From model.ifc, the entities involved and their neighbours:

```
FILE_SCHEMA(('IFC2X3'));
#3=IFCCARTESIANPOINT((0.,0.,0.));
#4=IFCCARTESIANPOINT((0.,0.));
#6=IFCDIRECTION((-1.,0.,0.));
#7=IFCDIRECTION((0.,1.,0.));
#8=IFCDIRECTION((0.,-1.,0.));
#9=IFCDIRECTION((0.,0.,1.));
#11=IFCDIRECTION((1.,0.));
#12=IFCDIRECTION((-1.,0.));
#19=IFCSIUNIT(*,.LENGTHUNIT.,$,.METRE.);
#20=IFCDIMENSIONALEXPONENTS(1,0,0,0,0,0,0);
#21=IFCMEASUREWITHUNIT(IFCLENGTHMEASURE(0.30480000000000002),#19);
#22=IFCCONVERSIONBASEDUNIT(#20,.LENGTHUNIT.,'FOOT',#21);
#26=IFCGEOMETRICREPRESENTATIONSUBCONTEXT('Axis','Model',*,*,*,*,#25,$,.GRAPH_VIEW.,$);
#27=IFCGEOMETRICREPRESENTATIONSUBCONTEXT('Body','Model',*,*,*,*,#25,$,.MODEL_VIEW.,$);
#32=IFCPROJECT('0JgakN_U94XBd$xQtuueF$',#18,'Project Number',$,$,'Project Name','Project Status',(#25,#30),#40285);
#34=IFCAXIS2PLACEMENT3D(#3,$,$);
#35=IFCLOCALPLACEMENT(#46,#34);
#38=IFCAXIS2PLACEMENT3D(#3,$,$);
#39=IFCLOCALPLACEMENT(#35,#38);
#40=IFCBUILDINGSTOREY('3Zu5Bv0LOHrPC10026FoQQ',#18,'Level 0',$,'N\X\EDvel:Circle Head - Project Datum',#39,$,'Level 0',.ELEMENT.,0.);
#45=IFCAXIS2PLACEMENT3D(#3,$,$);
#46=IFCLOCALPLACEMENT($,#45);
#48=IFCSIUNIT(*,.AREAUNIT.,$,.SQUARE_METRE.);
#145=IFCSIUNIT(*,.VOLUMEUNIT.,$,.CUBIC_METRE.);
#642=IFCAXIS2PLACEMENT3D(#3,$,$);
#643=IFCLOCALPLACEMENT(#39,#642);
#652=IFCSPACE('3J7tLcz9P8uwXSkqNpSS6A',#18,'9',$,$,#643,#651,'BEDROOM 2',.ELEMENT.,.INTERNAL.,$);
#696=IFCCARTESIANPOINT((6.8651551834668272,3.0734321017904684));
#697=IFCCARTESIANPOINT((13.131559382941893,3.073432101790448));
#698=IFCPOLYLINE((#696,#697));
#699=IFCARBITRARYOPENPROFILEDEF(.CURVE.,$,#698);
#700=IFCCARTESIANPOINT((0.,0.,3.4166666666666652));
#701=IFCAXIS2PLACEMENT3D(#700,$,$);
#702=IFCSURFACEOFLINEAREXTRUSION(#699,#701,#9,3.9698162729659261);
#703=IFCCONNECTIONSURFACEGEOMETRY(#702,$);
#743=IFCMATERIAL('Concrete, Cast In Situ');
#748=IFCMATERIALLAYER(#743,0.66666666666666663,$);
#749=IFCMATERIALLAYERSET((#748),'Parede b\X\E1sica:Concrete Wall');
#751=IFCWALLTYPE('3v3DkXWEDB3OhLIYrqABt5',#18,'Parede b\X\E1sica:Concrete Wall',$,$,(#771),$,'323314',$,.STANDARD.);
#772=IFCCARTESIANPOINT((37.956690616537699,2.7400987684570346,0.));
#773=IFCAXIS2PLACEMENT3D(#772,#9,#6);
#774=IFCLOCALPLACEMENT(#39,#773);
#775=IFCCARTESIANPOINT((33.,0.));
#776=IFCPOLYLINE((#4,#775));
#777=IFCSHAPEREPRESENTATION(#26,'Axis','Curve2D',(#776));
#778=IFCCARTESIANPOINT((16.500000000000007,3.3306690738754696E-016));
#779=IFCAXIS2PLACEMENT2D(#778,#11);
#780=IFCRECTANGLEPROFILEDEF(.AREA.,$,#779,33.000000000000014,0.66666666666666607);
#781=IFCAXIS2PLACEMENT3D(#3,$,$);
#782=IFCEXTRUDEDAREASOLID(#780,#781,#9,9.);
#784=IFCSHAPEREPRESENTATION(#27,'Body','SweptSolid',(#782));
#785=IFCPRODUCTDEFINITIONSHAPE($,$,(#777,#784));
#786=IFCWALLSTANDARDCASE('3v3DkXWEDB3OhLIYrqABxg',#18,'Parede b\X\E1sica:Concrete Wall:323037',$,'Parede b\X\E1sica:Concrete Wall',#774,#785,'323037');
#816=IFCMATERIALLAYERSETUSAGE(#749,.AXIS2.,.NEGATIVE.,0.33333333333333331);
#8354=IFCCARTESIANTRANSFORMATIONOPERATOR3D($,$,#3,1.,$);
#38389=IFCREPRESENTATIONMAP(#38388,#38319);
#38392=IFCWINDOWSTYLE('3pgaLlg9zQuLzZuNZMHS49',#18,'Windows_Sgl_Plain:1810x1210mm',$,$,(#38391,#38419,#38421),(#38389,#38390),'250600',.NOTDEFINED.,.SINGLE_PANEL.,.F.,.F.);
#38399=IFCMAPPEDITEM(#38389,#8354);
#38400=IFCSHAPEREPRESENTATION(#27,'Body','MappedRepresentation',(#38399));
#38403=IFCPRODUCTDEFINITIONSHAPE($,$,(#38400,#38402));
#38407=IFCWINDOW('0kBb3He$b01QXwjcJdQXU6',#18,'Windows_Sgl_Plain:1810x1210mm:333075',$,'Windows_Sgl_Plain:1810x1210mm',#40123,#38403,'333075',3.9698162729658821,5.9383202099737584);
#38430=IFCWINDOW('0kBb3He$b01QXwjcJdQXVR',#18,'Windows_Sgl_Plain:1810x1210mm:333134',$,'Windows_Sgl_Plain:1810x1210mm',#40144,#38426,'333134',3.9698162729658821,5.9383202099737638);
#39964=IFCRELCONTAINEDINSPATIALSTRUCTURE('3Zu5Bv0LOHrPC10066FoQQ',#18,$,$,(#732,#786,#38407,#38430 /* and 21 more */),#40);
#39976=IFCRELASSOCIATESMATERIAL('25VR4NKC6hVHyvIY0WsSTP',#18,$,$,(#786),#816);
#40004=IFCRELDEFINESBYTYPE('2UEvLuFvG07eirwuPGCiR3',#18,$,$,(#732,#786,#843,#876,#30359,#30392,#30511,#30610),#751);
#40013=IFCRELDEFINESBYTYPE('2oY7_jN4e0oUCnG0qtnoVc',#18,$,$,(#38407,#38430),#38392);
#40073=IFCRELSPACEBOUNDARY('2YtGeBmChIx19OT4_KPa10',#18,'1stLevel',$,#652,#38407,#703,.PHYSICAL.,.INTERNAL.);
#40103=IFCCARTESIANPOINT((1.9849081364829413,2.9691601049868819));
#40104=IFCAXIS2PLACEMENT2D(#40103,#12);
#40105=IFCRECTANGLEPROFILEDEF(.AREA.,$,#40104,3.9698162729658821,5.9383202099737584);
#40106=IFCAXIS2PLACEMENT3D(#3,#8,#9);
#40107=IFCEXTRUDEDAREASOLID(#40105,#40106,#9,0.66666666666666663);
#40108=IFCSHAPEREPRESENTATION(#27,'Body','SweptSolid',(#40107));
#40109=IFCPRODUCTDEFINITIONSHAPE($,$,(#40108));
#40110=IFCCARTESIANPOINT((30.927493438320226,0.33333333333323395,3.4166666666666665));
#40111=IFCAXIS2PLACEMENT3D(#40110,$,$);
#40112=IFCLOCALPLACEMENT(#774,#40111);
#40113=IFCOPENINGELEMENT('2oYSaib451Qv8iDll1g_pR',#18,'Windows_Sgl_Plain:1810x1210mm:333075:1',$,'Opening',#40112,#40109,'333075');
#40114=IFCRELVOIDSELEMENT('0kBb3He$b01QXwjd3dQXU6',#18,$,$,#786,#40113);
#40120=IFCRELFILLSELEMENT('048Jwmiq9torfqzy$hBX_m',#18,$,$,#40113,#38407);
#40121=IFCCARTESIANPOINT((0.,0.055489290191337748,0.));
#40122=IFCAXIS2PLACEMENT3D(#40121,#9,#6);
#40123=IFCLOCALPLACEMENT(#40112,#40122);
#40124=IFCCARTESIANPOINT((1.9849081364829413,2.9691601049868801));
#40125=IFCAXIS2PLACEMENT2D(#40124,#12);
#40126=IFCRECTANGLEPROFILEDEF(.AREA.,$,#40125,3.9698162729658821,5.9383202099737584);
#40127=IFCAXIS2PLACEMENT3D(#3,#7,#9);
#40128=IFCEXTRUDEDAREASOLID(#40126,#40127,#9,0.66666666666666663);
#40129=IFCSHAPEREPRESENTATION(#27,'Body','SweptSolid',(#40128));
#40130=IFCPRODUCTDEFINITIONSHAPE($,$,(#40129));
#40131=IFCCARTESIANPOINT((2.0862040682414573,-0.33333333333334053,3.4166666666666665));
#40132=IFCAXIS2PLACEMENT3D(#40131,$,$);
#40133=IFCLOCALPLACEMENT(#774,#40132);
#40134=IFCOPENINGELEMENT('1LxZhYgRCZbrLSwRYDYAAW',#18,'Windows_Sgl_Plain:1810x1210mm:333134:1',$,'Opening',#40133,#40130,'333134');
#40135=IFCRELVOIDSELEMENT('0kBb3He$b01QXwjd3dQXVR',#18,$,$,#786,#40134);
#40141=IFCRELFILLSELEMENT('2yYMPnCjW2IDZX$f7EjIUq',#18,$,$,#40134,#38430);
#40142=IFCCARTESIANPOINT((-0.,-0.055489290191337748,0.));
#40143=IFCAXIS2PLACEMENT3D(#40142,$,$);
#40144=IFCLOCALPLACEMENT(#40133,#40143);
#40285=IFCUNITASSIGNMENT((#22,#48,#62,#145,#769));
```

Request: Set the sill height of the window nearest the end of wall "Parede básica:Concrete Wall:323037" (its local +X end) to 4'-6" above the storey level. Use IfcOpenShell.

```python
import numpy as np
import ifcopenshell
import ifcopenshell.api.geometry
import ifcopenshell.geom
import ifcopenshell.util.element
import ifcopenshell.util.placement
import ifcopenshell.util.shape
import ifcopenshell.util.unit

model = ifcopenshell.open("model.ifc")
unit_scale = ifcopenshell.util.unit.calculate_unit_scale(model)

window = model.by_guid("0kBb3He$b01QXwjcJdQXU6")
opening = window.FillsVoids[0].RelatingOpeningElement
storey = ifcopenshell.util.element.get_container(window, ifc_class="IfcBuildingStorey")
level = ifcopenshell.util.placement.get_local_placement(storey.ObjectPlacement)[2, 3]

# The opening's origin need not be at the sill, so measure its lowest point.
shape = ifcopenshell.geom.create_shape(ifcopenshell.geom.settings(), opening)
bottom = ifcopenshell.util.shape.get_shape_bottom_elevation(shape, shape.geometry) / unit_scale
dz = level + 54 * 0.0254 / unit_scale - bottom

shift = np.array([0.0, 0.0, dz])
# The window is placed relative to its opening, so it follows when the opening moves.
matrix = ifcopenshell.util.placement.get_local_placement(opening.ObjectPlacement)
matrix[:3, 3] += shift
ifcopenshell.api.geometry.edit_object_placement(
    model, product=opening, matrix=matrix, is_si=False, should_transform_children=True
)

# Space boundary surfaces are stored in each space's coordinates; move them too.
for rel in window.ProvidesBoundaries:
    if not rel.ConnectionGeometry:
        continue
    surface = rel.ConnectionGeometry.SurfaceOnRelatingElement
    space_matrix = ifcopenshell.util.placement.get_local_placement(rel.RelatingSpace.ObjectPlacement)
    point = np.array(surface.Position.Location.Coordinates) + space_matrix[:3, :3].T @ shift
    surface.Position = model.createIfcAxis2Placement3D(
        model.createIfcCartesianPoint(point.tolist()), surface.Position.Axis, surface.Position.RefDirection
    )

print(f"moved by {dz * unit_scale:+.3f} m")

model.write("model_updated.ifc")
```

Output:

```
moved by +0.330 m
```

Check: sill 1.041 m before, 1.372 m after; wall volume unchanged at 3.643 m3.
